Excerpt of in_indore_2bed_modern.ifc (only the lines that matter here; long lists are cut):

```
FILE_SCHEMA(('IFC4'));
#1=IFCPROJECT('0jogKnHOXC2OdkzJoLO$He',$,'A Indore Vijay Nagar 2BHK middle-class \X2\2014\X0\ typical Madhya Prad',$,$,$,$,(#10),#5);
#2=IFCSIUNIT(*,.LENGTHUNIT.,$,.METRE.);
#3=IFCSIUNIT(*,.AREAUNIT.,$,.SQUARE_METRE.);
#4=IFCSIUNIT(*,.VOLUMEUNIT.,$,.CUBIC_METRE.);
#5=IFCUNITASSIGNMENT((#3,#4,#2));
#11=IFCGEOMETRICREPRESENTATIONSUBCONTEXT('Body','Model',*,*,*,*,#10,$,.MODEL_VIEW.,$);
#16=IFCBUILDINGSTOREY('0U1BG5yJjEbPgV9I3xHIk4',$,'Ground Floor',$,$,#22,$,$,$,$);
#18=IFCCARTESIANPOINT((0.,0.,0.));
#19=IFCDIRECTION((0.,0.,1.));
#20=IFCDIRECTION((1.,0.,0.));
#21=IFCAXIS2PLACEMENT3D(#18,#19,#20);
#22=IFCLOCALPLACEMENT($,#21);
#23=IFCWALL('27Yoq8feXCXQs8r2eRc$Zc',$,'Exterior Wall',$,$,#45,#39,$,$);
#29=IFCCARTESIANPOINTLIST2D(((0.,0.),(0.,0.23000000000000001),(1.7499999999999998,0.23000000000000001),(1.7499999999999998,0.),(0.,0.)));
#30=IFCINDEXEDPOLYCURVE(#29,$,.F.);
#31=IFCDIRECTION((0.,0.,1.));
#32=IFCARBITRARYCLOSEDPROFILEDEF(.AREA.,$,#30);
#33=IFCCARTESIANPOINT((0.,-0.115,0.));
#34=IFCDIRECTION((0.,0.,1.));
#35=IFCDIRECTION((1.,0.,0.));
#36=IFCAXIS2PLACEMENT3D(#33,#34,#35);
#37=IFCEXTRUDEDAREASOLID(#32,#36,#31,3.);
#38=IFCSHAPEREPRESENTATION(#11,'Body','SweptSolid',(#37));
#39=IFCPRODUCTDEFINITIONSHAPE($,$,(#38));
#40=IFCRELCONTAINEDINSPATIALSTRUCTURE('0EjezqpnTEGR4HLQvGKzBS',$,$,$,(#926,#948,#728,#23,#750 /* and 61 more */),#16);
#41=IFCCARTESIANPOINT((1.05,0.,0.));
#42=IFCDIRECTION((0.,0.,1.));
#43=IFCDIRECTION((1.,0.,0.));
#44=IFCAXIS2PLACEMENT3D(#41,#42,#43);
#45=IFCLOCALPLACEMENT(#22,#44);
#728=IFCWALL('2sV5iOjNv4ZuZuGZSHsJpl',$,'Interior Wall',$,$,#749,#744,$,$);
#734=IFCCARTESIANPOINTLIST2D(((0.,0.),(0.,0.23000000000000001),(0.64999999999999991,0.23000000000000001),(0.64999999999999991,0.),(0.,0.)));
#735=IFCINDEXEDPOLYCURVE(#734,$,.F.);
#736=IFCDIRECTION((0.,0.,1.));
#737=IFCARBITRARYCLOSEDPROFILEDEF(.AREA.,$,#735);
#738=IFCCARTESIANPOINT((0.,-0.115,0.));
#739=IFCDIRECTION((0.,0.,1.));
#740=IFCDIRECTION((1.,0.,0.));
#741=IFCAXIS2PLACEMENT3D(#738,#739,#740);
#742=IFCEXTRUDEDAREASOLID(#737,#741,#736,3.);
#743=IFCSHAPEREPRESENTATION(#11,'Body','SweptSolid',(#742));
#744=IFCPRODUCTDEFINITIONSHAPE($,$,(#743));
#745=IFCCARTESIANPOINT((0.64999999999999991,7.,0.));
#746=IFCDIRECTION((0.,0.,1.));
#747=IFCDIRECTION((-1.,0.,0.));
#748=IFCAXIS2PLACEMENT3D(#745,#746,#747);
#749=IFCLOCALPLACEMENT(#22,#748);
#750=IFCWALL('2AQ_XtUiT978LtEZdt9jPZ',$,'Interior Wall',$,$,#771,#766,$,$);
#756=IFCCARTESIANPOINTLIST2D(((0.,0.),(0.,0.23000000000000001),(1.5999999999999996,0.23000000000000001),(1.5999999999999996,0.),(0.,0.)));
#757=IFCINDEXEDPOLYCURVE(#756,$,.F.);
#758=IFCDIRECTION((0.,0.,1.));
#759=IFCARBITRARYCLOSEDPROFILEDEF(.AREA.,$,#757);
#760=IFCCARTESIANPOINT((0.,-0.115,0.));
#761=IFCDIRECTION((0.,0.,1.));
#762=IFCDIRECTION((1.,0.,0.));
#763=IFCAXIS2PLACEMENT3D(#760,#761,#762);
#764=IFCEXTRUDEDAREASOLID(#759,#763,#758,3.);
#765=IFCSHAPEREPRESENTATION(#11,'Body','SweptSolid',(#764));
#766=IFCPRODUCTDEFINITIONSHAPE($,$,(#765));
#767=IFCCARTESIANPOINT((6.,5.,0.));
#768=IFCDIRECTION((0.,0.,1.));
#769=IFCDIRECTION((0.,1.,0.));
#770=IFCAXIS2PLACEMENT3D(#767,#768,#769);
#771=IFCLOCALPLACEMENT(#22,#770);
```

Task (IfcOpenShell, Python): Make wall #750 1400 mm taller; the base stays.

```python
import ifcopenshell
import ifcopenshell.geom
import ifcopenshell.util.representation
import ifcopenshell.util.shape
import ifcopenshell.util.unit

model = ifcopenshell.open("in_indore_2bed_modern.ifc")
unit_scale = ifcopenshell.util.unit.calculate_unit_scale(model)
settings = ifcopenshell.geom.settings()


def volume(element):
    """Net volume in cubic metres, openings subtracted."""
    shape = ifcopenshell.geom.create_shape(settings, element)
    return ifcopenshell.util.shape.get_volume(shape.geometry)


wall = model.by_guid("2AQ_XtUiT978LtEZdt9jPZ")
before = volume(wall)

body = ifcopenshell.util.representation.get_representation(wall, "Model", "Body")
solid = body.Items[0]
old_height = solid.Depth
solid.Depth += 1.4 / unit_scale
after = volume(wall)

print(f"height {old_height:g} -> {solid.Depth:g}, volume {before:.3f} -> {after:.3f} m3")

model.write("in_indore_2bed_modern_rev.ifc")
```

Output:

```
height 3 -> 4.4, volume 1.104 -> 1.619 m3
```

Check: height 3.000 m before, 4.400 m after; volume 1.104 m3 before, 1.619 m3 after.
